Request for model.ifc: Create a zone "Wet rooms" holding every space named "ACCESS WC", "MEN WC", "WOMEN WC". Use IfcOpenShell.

First a look at what the model holds.

```python
import ifcopenshell

model = ifcopenshell.open("model.ifc")
print(model.schema)
seen = {}
for space in model.by_type("IfcSpace"):
    seen[space.LongName] = seen.get(space.LongName, 0) + 1
for name, count in sorted(seen.items(), key=str):
    print(count, "x", name)
print("zones:", [z.Name for z in model.by_type("IfcZone")][:20])
```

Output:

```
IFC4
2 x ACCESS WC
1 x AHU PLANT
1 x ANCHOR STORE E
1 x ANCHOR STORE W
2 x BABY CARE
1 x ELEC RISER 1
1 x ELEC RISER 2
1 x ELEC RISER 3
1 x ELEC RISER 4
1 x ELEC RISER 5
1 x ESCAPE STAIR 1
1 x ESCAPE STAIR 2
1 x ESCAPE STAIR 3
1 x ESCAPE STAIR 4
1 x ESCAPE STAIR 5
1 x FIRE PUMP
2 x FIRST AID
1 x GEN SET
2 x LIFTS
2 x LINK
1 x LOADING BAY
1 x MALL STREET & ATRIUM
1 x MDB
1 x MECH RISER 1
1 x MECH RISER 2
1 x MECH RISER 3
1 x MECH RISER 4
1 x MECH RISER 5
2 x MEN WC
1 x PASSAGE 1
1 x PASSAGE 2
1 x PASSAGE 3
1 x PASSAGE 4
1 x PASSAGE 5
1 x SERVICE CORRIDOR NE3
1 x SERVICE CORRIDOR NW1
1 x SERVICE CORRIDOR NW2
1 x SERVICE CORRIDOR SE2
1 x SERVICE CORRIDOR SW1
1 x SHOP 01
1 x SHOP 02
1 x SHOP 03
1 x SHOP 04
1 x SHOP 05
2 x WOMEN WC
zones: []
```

```python
import ifcopenshell
import ifcopenshell.api.group
import ifcopenshell.api.root

model = ifcopenshell.open("model.ifc")

names = {"ACCESS WC", "MEN WC", "WOMEN WC"}
spaces = [s for s in model.by_type("IfcSpace") if s.LongName in names]

zone = ifcopenshell.api.root.create_entity(model, ifc_class="IfcZone", name="Wet rooms")
ifcopenshell.api.group.assign_group(model, products=spaces, group=zone)
print(len(spaces), "spaces in", zone.Name)

model.write("model_rev.ifc")
```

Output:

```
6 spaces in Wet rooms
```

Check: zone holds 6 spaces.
